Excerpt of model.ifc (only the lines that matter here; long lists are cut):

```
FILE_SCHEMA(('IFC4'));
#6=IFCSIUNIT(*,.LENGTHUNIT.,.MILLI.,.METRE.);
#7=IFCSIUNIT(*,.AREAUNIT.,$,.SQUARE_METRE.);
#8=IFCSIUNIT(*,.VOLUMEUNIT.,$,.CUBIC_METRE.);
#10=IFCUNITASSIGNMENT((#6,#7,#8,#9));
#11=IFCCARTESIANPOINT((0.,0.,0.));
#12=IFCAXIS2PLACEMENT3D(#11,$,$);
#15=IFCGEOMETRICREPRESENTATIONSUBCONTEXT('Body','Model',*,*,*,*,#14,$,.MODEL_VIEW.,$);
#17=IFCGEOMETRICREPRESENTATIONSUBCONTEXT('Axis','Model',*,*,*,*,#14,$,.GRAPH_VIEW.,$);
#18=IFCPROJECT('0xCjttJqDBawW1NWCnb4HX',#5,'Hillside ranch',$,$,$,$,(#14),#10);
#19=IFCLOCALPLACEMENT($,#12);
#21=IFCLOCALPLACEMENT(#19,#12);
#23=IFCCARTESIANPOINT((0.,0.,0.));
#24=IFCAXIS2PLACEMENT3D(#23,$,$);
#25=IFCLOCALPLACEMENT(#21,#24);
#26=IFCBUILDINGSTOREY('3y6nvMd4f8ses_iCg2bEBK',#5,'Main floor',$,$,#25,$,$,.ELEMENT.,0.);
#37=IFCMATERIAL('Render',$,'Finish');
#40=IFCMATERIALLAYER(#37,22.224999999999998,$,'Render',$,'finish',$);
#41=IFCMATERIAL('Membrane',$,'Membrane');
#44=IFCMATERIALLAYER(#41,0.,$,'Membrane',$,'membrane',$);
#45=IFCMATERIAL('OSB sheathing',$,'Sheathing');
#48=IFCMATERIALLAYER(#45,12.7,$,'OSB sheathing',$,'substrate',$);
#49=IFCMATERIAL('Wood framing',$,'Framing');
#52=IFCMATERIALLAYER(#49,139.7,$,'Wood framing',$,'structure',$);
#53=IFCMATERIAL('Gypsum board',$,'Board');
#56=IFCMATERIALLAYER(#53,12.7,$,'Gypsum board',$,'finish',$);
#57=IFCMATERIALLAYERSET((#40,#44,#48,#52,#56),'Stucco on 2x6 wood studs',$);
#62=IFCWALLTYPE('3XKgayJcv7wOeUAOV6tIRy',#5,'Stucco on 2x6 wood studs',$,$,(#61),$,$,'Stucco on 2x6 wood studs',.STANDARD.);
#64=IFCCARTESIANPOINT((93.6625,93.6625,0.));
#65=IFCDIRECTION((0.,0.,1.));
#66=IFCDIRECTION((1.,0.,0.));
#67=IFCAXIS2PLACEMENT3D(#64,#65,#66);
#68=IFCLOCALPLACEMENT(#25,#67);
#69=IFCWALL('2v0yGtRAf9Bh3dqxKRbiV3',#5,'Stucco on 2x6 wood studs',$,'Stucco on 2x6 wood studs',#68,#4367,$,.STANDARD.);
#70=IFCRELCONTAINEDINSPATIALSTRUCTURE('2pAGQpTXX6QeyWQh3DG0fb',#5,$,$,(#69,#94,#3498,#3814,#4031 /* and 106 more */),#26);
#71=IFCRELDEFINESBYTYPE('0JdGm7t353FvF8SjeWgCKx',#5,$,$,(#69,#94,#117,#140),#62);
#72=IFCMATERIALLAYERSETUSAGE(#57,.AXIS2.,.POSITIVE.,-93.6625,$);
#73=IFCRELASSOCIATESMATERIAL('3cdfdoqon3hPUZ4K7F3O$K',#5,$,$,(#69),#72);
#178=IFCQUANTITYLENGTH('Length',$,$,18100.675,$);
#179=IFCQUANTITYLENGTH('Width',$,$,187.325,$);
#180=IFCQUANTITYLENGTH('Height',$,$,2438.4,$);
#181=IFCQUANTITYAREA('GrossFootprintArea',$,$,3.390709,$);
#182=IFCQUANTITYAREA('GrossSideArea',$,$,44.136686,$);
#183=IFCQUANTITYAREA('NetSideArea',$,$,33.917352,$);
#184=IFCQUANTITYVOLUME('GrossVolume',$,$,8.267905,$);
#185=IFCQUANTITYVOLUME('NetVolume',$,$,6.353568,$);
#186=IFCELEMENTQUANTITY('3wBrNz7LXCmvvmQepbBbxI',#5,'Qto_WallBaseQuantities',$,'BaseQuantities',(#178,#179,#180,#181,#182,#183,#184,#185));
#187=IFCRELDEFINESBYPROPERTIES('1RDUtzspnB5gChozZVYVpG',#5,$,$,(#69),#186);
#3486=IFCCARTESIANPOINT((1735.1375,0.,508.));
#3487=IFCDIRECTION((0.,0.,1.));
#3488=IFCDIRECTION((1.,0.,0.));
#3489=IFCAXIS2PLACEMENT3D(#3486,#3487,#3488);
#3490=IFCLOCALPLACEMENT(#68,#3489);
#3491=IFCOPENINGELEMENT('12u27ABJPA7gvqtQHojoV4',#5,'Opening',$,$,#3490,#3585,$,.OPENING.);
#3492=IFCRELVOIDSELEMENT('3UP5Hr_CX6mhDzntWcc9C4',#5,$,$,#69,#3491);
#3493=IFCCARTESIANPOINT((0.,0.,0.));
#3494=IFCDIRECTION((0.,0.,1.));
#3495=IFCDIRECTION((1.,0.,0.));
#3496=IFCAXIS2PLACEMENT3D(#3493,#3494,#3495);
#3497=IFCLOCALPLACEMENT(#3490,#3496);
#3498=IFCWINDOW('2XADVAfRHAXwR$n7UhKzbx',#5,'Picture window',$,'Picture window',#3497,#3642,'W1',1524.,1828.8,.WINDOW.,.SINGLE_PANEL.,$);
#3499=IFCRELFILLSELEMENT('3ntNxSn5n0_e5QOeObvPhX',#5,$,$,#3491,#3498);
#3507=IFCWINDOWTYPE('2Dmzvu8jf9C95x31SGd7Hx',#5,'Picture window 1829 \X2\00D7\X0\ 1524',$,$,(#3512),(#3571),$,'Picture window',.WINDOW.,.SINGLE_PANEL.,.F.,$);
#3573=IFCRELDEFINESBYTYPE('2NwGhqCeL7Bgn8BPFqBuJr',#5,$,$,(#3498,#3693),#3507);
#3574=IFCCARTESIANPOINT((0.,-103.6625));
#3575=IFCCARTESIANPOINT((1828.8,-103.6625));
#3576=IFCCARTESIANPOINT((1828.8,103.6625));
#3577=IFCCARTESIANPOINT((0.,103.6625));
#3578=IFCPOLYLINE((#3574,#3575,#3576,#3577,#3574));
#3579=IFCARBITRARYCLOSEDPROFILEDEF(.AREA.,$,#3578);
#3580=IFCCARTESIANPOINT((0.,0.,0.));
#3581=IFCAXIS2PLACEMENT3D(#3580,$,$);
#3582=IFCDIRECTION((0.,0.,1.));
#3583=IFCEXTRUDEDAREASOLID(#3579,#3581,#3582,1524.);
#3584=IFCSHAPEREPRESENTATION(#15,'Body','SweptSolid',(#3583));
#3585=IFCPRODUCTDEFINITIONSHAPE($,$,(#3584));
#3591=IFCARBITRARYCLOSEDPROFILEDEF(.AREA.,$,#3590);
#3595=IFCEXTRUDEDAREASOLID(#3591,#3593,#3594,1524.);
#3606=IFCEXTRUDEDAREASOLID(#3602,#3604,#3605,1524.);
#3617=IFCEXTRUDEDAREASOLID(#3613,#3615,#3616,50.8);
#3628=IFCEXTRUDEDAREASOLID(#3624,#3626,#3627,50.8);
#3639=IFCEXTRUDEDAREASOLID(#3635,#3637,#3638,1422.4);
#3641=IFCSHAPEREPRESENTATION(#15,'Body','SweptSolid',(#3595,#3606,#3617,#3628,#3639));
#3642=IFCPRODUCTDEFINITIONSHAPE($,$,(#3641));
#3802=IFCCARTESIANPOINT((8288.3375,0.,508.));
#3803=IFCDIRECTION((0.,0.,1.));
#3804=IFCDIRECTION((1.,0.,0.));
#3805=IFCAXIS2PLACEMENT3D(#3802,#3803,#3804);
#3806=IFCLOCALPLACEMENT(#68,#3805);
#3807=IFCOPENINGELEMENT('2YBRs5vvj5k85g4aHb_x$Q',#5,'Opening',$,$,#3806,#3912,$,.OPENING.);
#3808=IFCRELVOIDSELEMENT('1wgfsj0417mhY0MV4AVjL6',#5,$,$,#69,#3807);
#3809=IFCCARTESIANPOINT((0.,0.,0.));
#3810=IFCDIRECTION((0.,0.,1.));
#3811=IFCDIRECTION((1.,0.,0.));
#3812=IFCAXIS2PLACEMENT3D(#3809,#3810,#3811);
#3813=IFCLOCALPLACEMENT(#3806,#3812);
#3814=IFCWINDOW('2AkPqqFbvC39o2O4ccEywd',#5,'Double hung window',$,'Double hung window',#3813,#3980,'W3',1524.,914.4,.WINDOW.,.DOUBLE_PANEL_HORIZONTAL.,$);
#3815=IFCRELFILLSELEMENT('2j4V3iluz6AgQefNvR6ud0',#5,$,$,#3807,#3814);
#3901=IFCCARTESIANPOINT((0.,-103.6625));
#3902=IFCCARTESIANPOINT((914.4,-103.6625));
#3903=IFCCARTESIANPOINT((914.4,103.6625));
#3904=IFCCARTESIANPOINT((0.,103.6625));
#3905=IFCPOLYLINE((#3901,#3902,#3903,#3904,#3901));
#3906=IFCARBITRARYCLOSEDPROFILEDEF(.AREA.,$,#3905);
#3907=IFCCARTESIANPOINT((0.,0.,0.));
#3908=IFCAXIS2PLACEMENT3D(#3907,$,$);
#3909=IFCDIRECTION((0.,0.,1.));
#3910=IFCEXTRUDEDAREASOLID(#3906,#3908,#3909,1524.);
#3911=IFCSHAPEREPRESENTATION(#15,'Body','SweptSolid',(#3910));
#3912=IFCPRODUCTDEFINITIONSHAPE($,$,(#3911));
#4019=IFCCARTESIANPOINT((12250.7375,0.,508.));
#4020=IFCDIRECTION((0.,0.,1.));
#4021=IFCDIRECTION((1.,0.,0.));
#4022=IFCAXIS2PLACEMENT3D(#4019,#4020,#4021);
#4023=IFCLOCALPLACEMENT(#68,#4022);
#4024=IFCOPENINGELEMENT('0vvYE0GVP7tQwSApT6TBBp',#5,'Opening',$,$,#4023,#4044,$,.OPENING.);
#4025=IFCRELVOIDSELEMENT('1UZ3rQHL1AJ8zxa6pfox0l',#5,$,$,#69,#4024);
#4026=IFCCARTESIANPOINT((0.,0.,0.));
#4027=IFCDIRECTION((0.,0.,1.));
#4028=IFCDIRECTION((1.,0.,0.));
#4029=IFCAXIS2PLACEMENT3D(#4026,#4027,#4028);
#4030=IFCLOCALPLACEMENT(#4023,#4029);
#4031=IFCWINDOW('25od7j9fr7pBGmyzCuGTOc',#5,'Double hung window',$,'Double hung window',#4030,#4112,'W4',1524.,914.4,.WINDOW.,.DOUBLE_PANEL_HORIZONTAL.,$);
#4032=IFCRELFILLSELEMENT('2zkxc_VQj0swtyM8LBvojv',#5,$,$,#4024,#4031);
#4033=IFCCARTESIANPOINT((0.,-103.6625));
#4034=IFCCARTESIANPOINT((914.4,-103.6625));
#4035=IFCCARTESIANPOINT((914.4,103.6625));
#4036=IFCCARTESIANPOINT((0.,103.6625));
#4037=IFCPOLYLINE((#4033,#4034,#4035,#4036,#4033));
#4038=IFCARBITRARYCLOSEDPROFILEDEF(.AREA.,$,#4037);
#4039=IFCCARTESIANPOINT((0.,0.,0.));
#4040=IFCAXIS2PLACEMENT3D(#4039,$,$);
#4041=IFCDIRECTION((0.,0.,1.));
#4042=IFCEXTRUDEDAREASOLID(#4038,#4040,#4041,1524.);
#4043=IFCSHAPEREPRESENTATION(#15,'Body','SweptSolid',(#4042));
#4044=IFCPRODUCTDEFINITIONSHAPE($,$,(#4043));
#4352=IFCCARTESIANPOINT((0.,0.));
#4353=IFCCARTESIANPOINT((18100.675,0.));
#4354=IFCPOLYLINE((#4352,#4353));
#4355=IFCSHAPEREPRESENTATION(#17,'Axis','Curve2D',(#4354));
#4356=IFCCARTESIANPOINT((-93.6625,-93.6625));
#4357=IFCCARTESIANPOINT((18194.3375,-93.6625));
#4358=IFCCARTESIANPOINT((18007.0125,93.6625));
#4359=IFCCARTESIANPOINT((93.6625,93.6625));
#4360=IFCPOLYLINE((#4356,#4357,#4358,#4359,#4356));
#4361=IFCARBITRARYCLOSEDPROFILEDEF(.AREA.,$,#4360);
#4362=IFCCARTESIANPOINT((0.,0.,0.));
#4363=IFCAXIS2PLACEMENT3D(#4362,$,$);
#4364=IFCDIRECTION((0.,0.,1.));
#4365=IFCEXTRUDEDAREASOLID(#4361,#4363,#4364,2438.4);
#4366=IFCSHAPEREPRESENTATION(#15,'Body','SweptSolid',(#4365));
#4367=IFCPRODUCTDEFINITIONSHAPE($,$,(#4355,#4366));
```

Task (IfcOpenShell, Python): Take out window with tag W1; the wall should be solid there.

```python
import ifcopenshell
import ifcopenshell.api.feature
import ifcopenshell.api.pset
import ifcopenshell.api.root
import ifcopenshell.geom
import ifcopenshell.util.element
import ifcopenshell.util.shape
import ifcopenshell.util.unit

model = ifcopenshell.open("model.ifc")
area_scale = ifcopenshell.util.unit.calculate_unit_scale(model, "AREAUNIT")
volume_scale = ifcopenshell.util.unit.calculate_unit_scale(model, "VOLUMEUNIT")
settings = ifcopenshell.geom.settings()


def volume(element):
    """Net volume in cubic metres, openings subtracted."""
    shape = ifcopenshell.geom.create_shape(settings, element)
    return ifcopenshell.util.shape.get_volume(shape.geometry)


window = model.by_guid("2XADVAfRHAXwR$n7UhKzbx")
opening = window.FillsVoids[0].RelatingOpeningElement
wall = opening.VoidsElements[0].RelatingBuildingElement
before = volume(wall)

ifcopenshell.api.root.remove_product(model, product=window)
ifcopenshell.api.feature.remove_feature(model, feature=opening)

after = volume(wall)
thickness = 0.1873  # wall thickness in metres

# Update the wall's stored quantities.
qto = model.by_id(ifcopenshell.util.element.get_pset(wall, "Qto_WallBaseQuantities", should_inherit=False)["id"])
ifcopenshell.api.pset.edit_qto(model, qto=qto, properties={
    "NetSideArea": after / thickness / area_scale,
    "NetVolume": after / volume_scale,
})

print(f"wall volume {before:.3f} -> {after:.3f} m3")

model.write("model_updated.ifc")
```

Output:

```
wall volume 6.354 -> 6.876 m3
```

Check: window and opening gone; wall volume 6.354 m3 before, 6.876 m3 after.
